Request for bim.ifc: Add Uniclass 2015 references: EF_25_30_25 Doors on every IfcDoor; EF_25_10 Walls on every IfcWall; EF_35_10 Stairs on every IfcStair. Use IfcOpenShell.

First a look at what the model holds.

```python
import ifcopenshell

model = ifcopenshell.open("bim.ifc")
print(model.schema)
print("classifications:", [c.Name for c in model.by_type("IfcClassification")])
for ifc_class in ("IfcDoor", "IfcRoof", "IfcStair", "IfcWall", "IfcWindow"):
    print(ifc_class, len(model.by_type(ifc_class)))
```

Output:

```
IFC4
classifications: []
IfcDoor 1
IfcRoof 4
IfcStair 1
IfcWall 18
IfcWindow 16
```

```python
import ifcopenshell
import ifcopenshell.api.classification

model = ifcopenshell.open("bim.ifc")

system = ifcopenshell.api.classification.add_classification(model, classification="Uniclass 2015")

codes = {
    "IfcDoor": ("EF_25_30_25", "Doors"),
    "IfcWall": ("EF_25_10", "Walls"),
    "IfcStair": ("EF_35_10", "Stairs"),
}
for ifc_class, (code, name) in codes.items():
    products = model.by_type(ifc_class)
    ifcopenshell.api.classification.add_reference(
        model, products=products, classification=system, identification=code, name=name
    )
    print(code, len(products))

model.write("bim_updated.ifc")
```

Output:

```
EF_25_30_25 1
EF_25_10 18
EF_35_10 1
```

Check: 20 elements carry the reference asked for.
